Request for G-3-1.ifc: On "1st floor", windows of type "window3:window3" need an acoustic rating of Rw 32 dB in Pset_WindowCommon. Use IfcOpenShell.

First a look at what the model holds.

```python
import ifcopenshell
import ifcopenshell.util.element

model = ifcopenshell.open("G-3-1.ifc")
print(model.schema)
storey = next(s for s in model.by_type("IfcBuildingStorey") if s.Name == "1st floor")
windows = [e for e in ifcopenshell.util.element.get_decomposition(storey) if e.is_a("IfcWindow")]
seen = {}
for e in windows:
    element_type = ifcopenshell.util.element.get_type(e)
    key = (element_type.Name if element_type != e and element_type else None, ifcopenshell.util.element.get_pset(e, "Pset_WindowCommon", "AcousticRating"))
    seen[key] = seen.get(key, 0) + 1
for (name, value), count in sorted(seen.items(), key=str):
    print(count, "x", name, "|", value)
```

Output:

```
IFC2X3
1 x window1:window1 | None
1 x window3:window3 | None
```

```python
import ifcopenshell
import ifcopenshell.api.pset
import ifcopenshell.util.element

model = ifcopenshell.open("G-3-1.ifc")

storey = next(s for s in model.by_type("IfcBuildingStorey") if s.Name == "1st floor")
windows = [e for e in ifcopenshell.util.element.get_decomposition(storey) if e.is_a("IfcWindow")]

count = 0
for e in windows:
    element_type = ifcopenshell.util.element.get_type(e)
    if element_type in (None, e) or element_type.Name != "window3:window3":
        continue
    # add_pset returns the element's existing set when there is one.
    pset = ifcopenshell.api.pset.add_pset(model, product=e, name="Pset_WindowCommon")
    ifcopenshell.api.pset.edit_pset(model, pset=pset, properties={"AcousticRating": "Rw 32 dB"})
    count += 1

print(count, "windows updated")

model.write("G-3-1_v2.ifc")
```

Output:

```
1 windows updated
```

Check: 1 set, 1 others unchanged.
